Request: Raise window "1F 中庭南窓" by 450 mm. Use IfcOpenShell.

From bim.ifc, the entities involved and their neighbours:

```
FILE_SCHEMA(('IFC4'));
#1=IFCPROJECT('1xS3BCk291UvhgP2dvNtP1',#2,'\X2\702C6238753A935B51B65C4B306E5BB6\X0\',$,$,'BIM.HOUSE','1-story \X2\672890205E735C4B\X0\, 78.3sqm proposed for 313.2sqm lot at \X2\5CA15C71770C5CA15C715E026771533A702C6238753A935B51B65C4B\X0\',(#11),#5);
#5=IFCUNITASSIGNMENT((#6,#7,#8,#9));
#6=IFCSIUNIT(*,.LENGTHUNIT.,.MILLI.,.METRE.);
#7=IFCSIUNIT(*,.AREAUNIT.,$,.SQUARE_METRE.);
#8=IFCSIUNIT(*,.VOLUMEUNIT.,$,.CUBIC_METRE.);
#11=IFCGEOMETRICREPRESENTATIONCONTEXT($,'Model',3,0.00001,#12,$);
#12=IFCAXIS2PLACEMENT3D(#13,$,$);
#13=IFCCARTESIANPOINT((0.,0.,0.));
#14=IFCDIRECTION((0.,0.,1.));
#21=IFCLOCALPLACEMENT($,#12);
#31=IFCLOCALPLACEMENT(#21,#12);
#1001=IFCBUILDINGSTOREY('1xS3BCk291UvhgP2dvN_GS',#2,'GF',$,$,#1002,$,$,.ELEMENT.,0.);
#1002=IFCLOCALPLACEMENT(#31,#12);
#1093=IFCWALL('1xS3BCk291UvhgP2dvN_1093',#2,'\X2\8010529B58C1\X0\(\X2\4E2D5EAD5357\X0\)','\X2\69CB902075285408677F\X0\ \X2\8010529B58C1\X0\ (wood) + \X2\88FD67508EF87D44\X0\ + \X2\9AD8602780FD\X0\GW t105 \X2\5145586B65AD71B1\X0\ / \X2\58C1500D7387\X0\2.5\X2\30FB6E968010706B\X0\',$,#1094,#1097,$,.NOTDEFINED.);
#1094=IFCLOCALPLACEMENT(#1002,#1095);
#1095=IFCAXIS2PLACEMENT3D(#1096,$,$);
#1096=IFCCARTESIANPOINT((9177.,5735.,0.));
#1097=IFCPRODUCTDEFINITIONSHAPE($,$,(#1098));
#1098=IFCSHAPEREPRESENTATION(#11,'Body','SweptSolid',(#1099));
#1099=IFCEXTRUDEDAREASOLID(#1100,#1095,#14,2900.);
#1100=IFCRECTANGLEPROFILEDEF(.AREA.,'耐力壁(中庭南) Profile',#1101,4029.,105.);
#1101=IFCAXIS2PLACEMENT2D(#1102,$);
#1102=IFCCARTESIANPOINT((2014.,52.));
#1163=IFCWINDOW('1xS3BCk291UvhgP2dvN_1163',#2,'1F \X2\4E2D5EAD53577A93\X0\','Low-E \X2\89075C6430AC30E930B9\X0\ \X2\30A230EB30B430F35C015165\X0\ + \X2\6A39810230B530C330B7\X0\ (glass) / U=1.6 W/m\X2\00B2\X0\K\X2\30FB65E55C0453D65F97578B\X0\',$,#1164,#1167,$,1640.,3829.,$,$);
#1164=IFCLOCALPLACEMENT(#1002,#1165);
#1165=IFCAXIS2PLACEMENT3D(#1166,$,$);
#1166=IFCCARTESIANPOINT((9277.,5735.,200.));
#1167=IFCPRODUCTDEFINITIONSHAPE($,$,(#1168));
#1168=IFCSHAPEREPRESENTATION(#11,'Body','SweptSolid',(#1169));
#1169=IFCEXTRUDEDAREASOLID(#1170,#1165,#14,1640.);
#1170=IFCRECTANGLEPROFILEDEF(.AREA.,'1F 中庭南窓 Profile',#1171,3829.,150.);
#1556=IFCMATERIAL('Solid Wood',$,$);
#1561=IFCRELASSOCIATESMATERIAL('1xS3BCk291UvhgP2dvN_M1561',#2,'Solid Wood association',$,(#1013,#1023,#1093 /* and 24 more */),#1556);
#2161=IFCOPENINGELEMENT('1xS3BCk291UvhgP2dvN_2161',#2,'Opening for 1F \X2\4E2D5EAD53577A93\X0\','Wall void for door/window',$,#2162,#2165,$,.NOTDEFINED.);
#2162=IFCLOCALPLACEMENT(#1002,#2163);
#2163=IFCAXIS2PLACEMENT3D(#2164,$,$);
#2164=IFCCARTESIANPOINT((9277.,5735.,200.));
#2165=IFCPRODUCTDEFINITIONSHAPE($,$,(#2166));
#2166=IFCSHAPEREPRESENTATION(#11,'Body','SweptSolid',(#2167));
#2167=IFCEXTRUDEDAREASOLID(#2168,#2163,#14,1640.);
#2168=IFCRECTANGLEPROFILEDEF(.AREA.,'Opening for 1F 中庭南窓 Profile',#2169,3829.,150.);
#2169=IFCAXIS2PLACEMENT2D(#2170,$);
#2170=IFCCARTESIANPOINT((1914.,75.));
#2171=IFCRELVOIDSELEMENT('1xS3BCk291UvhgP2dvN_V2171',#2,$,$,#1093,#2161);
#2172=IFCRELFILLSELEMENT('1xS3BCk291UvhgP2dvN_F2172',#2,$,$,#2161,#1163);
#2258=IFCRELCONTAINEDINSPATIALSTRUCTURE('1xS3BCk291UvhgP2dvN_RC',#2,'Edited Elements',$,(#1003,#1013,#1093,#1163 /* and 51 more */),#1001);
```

```python
import numpy as np
import ifcopenshell
import ifcopenshell.api.geometry
import ifcopenshell.util.placement
import ifcopenshell.util.unit

model = ifcopenshell.open("bim.ifc")
unit_scale = ifcopenshell.util.unit.calculate_unit_scale(model)

window = model.by_guid("1xS3BCk291UvhgP2dvN_1163")
opening = window.FillsVoids[0].RelatingOpeningElement
dz = 450.0

shift = np.array([0.0, 0.0, dz])
# The window is not placed relative to its opening, so move both.
for product in (opening, window):
    matrix = ifcopenshell.util.placement.get_local_placement(product.ObjectPlacement)
    matrix[:3, 3] += shift
    ifcopenshell.api.geometry.edit_object_placement(model, product=product, matrix=matrix, is_si=False)

print(f"moved by {dz * unit_scale:+.3f} m")

model.write("bim_v2.ifc")
```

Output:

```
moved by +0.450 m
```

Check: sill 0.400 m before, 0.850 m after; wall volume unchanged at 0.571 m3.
